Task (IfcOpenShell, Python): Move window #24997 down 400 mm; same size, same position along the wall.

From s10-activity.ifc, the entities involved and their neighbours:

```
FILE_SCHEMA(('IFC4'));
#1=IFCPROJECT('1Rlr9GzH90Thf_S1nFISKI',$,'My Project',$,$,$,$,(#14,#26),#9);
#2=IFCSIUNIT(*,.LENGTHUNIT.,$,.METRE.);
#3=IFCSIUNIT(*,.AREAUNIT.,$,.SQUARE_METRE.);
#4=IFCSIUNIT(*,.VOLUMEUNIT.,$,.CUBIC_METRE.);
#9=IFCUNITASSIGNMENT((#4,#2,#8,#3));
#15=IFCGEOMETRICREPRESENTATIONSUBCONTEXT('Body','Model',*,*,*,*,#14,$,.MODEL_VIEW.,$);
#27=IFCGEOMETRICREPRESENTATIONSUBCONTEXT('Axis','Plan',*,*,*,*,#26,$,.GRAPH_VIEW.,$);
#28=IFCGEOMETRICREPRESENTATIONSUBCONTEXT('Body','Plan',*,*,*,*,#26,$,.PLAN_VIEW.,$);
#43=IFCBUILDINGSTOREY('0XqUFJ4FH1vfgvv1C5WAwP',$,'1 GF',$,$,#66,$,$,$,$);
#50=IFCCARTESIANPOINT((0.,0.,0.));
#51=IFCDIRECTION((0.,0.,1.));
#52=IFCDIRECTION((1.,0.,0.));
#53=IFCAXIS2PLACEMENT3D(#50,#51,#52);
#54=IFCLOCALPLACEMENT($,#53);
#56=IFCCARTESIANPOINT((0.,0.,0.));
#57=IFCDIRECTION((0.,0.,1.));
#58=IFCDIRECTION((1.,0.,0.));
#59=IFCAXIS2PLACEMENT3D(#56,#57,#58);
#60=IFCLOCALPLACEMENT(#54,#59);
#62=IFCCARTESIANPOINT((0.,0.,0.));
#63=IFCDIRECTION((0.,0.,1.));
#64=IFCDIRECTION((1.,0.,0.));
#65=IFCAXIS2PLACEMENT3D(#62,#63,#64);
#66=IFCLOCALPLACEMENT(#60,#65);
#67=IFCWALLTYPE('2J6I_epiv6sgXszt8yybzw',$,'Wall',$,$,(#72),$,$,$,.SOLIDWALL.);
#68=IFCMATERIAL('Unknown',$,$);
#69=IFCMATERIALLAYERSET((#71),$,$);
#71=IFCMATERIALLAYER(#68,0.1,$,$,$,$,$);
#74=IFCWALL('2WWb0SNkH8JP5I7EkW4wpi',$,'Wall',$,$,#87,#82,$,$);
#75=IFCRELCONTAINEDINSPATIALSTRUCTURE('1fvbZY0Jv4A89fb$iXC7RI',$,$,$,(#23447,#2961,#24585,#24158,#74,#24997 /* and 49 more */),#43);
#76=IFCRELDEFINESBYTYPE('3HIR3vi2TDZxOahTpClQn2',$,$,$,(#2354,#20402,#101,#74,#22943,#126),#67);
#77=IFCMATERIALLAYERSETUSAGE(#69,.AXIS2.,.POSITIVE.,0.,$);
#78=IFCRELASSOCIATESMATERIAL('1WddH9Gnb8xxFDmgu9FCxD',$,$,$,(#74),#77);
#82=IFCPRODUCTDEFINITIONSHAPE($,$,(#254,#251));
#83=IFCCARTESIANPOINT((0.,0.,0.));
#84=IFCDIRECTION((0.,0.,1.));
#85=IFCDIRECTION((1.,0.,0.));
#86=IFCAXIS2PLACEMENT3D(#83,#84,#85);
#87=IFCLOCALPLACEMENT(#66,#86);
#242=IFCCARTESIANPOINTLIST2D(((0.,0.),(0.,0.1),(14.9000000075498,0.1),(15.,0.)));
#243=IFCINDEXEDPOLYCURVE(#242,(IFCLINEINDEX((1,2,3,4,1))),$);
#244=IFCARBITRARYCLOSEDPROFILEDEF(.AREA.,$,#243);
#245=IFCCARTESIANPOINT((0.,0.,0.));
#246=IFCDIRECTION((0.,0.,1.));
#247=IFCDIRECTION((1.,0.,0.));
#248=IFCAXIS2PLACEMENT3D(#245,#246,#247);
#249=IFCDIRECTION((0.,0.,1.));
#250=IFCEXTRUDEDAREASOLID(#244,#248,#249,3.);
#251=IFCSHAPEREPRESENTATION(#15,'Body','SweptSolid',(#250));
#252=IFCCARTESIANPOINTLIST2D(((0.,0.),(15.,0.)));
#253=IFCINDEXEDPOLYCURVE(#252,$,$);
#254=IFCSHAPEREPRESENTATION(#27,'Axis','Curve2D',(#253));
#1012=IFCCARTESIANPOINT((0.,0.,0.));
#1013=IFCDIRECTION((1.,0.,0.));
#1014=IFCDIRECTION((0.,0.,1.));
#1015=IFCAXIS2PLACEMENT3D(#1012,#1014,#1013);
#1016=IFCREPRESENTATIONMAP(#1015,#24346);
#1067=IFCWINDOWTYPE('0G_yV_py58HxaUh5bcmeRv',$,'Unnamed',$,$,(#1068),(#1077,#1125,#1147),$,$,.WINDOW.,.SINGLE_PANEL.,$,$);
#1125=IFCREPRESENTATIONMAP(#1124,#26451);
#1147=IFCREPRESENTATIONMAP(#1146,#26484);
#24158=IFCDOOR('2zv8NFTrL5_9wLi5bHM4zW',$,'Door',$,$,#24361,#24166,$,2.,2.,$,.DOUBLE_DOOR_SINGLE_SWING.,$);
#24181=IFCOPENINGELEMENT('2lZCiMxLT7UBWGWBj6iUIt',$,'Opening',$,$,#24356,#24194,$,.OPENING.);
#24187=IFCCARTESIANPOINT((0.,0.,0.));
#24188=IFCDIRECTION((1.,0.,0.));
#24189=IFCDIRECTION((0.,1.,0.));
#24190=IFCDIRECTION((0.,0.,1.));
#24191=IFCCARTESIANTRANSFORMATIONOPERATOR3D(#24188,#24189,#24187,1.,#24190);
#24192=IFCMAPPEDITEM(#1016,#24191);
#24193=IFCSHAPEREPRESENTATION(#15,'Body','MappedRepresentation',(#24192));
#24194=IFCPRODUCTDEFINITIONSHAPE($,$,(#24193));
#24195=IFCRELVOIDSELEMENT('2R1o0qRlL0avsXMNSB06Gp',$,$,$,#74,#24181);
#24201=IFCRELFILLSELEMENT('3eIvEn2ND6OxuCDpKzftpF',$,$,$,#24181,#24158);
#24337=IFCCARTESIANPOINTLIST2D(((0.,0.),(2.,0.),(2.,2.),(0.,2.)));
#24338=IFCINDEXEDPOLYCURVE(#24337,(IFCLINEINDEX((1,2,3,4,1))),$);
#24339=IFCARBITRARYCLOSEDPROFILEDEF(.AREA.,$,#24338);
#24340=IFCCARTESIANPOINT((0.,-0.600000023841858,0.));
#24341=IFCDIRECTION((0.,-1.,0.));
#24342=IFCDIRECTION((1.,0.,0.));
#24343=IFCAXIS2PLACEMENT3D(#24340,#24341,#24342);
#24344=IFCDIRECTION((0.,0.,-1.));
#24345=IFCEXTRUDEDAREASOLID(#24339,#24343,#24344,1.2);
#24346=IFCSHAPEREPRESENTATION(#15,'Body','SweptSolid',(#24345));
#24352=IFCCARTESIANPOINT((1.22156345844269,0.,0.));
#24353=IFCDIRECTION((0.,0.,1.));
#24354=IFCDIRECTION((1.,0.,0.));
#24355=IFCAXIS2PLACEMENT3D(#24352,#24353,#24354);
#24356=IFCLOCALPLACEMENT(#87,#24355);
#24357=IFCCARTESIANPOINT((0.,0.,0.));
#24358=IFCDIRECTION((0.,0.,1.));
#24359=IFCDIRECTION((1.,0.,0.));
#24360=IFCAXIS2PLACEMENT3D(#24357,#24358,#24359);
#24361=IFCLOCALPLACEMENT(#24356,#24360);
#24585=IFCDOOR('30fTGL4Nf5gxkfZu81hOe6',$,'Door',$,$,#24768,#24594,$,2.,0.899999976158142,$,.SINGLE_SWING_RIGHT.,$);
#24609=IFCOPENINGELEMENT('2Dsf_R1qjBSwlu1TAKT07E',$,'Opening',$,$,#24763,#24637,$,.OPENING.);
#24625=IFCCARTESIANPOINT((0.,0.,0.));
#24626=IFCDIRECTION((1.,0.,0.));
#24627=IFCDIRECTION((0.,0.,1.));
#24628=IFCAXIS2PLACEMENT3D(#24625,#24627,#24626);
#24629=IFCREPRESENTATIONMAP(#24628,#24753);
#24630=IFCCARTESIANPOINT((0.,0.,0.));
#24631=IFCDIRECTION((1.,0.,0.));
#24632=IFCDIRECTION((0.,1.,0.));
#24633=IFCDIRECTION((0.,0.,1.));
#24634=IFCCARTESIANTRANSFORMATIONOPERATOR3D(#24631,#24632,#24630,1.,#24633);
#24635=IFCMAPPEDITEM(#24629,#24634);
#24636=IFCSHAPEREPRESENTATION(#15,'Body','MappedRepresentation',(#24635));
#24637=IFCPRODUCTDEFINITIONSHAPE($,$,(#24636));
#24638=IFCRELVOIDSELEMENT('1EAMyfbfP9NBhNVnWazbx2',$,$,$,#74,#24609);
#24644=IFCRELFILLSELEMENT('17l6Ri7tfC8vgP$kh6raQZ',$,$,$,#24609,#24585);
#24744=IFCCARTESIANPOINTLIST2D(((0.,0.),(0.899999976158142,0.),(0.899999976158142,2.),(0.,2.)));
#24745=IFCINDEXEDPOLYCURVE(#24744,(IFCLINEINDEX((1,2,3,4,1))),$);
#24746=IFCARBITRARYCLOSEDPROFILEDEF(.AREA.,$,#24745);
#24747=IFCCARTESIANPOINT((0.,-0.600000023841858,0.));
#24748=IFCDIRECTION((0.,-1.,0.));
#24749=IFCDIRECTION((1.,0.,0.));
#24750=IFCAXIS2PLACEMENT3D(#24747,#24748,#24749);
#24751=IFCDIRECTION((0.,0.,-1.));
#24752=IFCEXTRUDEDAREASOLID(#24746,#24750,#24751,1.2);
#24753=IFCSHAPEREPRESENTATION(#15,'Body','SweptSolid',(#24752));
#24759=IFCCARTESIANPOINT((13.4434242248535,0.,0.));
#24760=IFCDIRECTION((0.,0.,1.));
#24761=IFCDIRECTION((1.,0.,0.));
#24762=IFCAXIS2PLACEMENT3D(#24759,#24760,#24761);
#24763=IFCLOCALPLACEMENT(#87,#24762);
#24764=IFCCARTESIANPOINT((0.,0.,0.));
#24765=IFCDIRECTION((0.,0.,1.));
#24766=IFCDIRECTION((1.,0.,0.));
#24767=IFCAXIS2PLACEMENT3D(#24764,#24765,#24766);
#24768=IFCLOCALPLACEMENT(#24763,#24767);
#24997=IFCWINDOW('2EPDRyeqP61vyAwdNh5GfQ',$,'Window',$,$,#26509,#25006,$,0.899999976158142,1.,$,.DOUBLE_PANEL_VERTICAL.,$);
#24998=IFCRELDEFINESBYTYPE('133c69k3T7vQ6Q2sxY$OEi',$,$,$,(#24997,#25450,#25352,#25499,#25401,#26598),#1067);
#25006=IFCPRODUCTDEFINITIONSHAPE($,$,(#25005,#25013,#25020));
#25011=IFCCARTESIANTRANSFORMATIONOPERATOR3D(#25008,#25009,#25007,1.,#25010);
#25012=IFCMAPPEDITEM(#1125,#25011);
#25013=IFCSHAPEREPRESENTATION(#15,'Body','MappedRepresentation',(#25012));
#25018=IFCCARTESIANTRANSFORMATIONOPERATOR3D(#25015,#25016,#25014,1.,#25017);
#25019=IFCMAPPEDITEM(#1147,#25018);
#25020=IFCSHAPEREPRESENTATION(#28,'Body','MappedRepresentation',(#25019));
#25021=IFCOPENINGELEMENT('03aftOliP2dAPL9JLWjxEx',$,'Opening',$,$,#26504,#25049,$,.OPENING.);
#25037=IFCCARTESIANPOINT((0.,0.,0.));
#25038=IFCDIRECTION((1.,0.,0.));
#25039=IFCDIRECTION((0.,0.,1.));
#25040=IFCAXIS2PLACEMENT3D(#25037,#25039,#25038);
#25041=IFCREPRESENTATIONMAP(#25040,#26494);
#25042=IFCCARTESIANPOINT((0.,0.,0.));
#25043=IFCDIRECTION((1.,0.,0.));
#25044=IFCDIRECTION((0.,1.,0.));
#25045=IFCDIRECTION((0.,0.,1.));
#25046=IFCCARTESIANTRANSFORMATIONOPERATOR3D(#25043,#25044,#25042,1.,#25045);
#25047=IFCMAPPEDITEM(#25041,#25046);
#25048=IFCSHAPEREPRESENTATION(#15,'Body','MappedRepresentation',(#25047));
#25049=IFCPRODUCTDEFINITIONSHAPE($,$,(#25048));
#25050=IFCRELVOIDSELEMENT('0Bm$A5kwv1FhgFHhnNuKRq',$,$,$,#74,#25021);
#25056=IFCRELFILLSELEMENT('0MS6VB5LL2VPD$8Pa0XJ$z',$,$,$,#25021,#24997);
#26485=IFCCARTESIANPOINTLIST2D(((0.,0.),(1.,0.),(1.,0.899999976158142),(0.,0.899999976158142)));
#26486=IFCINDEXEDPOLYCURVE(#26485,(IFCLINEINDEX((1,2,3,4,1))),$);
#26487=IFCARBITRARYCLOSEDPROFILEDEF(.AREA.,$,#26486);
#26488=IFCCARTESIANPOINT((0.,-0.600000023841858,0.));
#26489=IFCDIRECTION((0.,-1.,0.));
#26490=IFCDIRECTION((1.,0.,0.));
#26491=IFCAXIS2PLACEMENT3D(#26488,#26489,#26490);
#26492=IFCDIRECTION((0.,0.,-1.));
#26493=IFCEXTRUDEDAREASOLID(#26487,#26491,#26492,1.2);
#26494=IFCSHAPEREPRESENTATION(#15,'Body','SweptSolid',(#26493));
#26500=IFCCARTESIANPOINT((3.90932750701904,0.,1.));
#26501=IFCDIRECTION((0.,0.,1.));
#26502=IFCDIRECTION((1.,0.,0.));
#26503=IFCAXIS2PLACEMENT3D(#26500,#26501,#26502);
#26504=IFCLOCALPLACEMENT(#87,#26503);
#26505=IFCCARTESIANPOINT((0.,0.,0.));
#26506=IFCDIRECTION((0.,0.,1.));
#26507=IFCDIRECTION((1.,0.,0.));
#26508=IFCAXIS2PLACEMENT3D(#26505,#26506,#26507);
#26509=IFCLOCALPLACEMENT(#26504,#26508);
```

```python
import numpy as np
import ifcopenshell
import ifcopenshell.api.geometry
import ifcopenshell.util.placement
import ifcopenshell.util.unit

model = ifcopenshell.open("s10-activity.ifc")
unit_scale = ifcopenshell.util.unit.calculate_unit_scale(model)

window = model.by_id(24997)
opening = window.FillsVoids[0].RelatingOpeningElement
dz = -0.4 / unit_scale

shift = np.array([0.0, 0.0, dz])
# The window is placed relative to its opening, so it follows when the opening moves.
matrix = ifcopenshell.util.placement.get_local_placement(opening.ObjectPlacement)
matrix[:3, 3] += shift
ifcopenshell.api.geometry.edit_object_placement(
    model, product=opening, matrix=matrix, is_si=False, should_transform_children=True
)

print(f"moved by {dz * unit_scale:+.3f} m")

model.write("s10-activity_edited.ifc")
```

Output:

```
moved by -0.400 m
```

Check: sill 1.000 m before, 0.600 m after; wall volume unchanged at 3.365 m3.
